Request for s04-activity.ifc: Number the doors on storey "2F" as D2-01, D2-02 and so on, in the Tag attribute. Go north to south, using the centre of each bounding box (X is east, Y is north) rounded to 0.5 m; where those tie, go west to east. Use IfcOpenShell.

First a look at what the model holds.

```python
import ifcopenshell
import ifcopenshell.util.element
import ifcopenshell.util.placement

model = ifcopenshell.open("s04-activity.ifc")
print(model.schema)
storey = next(s for s in model.by_type("IfcBuildingStorey") if s.Name == "2F")
doors = [e for e in ifcopenshell.util.element.get_decomposition(storey) if e.is_a("IfcDoor")]
for e in sorted(doors, key=lambda e: e.id()):
    origin = ifcopenshell.util.placement.get_local_placement(e.ObjectPlacement)[:3, 3]
    print(e.id(), e.Tag, e.Name, origin.round(2) + 0.0, sep=" | ")
```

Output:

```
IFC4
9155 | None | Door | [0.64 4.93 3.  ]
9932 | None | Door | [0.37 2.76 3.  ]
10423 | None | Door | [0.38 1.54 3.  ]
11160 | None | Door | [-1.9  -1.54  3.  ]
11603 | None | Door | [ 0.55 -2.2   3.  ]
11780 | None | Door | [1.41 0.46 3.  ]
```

```python
import ifcopenshell
import ifcopenshell.geom
import ifcopenshell.util.element
import ifcopenshell.util.shape

model = ifcopenshell.open("s04-activity.ifc")
settings = ifcopenshell.geom.settings()
settings.set("use-world-coords", True)


def centre(element):
    shape = ifcopenshell.geom.create_shape(settings, element)
    return ifcopenshell.util.shape.get_bbox_centroid(shape.geometry)


storey = next(s for s in model.by_type("IfcBuildingStorey") if s.Name == "2F")
doors = [e for e in ifcopenshell.util.element.get_decomposition(storey) if e.is_a("IfcDoor")]

# Insertion points can sit at a corner or the storey origin, so sort by the geometry (in metres).
centres = {e: centre(e) for e in doors}
doors.sort(key=lambda e: (-round(centres[e][1] / 0.5), centres[e][0]))

for i, e in enumerate(doors, start=1):
    number = f"D2-{i:02d}"
    e.Tag = number
    print(e.id(), number)

model.write("s04-activity_edited.ifc")
```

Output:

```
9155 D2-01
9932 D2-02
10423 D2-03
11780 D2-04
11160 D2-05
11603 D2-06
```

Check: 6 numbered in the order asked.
